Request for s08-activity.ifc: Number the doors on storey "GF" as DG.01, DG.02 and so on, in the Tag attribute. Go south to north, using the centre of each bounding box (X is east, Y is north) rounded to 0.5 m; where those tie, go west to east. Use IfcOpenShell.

First a look at what the model holds.

```python
import ifcopenshell
import ifcopenshell.util.element
import ifcopenshell.util.placement

model = ifcopenshell.open("s08-activity.ifc")
print(model.schema)
storey = next(s for s in model.by_type("IfcBuildingStorey") if s.Name == "GF")
doors = [e for e in ifcopenshell.util.element.get_decomposition(storey) if e.is_a("IfcDoor")]
for e in sorted(doors, key=lambda e: e.id()):
    origin = ifcopenshell.util.placement.get_local_placement(e.ObjectPlacement)[:3, 3]
    print(e.id(), e.Tag, e.Name, origin.round(2) + 0.0, sep=" | ")
```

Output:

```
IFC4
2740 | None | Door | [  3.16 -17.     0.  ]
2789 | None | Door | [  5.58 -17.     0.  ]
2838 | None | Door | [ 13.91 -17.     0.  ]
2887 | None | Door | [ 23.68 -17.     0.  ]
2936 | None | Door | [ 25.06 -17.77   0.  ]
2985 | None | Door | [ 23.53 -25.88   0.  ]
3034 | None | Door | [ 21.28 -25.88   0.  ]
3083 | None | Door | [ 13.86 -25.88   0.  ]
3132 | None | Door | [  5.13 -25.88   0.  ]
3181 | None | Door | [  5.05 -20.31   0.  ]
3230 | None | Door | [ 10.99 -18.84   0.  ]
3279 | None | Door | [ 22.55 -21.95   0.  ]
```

```python
import ifcopenshell
import ifcopenshell.geom
import ifcopenshell.util.element
import ifcopenshell.util.shape

model = ifcopenshell.open("s08-activity.ifc")
settings = ifcopenshell.geom.settings()
settings.set("use-world-coords", True)


def centre(element):
    shape = ifcopenshell.geom.create_shape(settings, element)
    return ifcopenshell.util.shape.get_bbox_centroid(shape.geometry)


storey = next(s for s in model.by_type("IfcBuildingStorey") if s.Name == "GF")
doors = [e for e in ifcopenshell.util.element.get_decomposition(storey) if e.is_a("IfcDoor")]

# Insertion points can sit at a corner or the storey origin, so sort by the geometry (in metres).
centres = {e: centre(e) for e in doors}
doors.sort(key=lambda e: (round(centres[e][1] / 0.5), centres[e][0]))

for i, e in enumerate(doors, start=1):
    number = f"DG.{i:02d}"
    e.Tag = number
    print(e.id(), number)

model.write("s08-activity_rev.ifc")
```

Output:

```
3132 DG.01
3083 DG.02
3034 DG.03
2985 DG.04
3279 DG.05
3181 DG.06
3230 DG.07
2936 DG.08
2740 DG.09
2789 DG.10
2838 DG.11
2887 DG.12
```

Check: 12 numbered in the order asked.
